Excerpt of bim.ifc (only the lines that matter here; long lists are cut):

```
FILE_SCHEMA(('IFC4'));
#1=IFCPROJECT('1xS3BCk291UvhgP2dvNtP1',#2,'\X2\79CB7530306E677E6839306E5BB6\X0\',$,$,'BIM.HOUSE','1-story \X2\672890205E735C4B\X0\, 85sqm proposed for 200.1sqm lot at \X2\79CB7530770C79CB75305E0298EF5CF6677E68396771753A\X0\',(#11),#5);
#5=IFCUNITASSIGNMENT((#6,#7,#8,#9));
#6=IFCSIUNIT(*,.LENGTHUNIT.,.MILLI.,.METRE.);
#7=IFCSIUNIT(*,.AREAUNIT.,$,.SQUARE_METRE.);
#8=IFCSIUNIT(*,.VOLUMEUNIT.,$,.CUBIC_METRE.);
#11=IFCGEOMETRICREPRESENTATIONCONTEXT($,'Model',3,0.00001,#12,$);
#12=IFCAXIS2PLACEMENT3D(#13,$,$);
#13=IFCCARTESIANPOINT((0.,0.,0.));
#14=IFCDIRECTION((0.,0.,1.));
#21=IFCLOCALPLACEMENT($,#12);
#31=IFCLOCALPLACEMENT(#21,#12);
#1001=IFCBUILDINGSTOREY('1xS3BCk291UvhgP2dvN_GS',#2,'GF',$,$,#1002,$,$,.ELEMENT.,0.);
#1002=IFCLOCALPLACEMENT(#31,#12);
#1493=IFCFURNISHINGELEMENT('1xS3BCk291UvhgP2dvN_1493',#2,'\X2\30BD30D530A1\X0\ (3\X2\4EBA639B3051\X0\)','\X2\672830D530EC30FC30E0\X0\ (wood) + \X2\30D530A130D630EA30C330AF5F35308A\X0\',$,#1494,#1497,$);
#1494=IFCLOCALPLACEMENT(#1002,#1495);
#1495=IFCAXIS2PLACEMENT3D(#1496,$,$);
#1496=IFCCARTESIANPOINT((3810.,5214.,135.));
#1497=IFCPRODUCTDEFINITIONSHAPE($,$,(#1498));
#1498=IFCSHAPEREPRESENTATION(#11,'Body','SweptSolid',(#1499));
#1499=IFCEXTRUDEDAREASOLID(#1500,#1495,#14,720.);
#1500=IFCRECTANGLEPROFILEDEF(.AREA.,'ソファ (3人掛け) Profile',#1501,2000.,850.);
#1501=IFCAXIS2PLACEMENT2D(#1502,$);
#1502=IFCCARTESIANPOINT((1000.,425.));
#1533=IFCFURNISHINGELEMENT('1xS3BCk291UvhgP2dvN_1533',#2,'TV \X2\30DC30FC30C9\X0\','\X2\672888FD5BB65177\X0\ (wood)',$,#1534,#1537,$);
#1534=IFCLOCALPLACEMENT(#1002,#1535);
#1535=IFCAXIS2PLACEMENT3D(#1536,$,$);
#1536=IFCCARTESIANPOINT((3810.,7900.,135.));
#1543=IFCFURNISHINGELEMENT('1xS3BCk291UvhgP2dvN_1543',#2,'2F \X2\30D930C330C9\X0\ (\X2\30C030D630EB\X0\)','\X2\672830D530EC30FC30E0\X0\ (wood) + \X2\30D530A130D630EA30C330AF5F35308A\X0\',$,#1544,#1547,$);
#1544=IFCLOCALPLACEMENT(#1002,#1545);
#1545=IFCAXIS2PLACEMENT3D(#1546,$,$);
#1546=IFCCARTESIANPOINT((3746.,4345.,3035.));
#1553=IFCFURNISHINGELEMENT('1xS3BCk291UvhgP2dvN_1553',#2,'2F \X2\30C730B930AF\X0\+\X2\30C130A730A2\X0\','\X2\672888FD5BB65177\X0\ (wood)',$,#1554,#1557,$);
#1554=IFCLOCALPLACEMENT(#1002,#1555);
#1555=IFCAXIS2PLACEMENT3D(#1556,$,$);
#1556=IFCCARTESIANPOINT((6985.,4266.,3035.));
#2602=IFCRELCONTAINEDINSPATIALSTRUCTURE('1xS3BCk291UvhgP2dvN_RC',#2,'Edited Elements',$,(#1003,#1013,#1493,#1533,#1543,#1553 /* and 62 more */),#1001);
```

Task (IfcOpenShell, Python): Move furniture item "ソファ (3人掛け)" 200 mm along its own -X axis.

```python
import ifcopenshell
import ifcopenshell.api.geometry
import ifcopenshell.util.placement
import ifcopenshell.util.unit

model = ifcopenshell.open("bim.ifc")
unit_scale = ifcopenshell.util.unit.calculate_unit_scale(model)

item = model.by_id(1493)
matrix = ifcopenshell.util.placement.get_local_placement(item.ObjectPlacement)
matrix[:3, 3] -= matrix[:3, 0] * 0.2 / unit_scale
ifcopenshell.api.geometry.edit_object_placement(model, product=item, matrix=matrix, is_si=False)

print(ifcopenshell.util.placement.get_local_placement(item.ObjectPlacement).round(3) + 0.0)

model.write("bim-out.ifc")
```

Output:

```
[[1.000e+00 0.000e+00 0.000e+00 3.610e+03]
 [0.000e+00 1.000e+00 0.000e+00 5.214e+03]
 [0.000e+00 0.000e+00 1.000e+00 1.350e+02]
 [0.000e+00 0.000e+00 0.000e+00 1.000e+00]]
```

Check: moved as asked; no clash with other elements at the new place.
